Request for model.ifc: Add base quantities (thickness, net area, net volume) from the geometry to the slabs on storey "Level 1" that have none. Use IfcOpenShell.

First a look at what the model holds.

```python
import ifcopenshell
import ifcopenshell.util.element
import ifcopenshell.util.unit

model = ifcopenshell.open("model.ifc")
print(model.schema)
for unit_type in ("LENGTHUNIT", "AREAUNIT", "VOLUMEUNIT"):
    print(unit_type, ifcopenshell.util.unit.calculate_unit_scale(model, unit_type))
storey = next(s for s in model.by_type("IfcBuildingStorey") if s.Name == "Level 1")
slabs = [e for e in ifcopenshell.util.element.get_decomposition(storey) if e.is_a("IfcSlab")]
for e in sorted(slabs, key=lambda e: e.id()):
    print(e.id(), e.is_a(), e.Name, list(ifcopenshell.util.element.get_psets(e, qtos_only=True)), sep=" | ")
```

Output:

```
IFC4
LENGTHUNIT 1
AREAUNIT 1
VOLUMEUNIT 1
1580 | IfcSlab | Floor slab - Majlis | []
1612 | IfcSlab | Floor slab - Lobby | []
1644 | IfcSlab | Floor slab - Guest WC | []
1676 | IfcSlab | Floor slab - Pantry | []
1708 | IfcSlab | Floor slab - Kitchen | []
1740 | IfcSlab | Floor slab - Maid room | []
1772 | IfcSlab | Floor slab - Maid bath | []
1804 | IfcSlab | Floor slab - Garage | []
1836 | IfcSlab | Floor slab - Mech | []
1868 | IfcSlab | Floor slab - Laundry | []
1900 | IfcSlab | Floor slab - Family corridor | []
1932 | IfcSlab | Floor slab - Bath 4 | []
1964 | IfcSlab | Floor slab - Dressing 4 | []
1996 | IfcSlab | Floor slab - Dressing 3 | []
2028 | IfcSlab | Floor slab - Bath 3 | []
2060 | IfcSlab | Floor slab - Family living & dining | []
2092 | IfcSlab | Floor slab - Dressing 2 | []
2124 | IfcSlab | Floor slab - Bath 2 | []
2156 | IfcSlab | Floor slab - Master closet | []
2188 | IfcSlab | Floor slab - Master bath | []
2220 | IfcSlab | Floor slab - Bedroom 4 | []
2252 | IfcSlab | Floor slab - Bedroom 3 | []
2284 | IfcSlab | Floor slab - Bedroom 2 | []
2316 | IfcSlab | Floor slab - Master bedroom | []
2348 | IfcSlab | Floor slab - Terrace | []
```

```python
import ifcopenshell
import ifcopenshell.api.pset
import ifcopenshell.geom
import ifcopenshell.util.element
import ifcopenshell.util.shape
import ifcopenshell.util.unit

model = ifcopenshell.open("model.ifc")
unit_scale = ifcopenshell.util.unit.calculate_unit_scale(model)
area_scale = ifcopenshell.util.unit.calculate_unit_scale(model, "AREAUNIT")
volume_scale = ifcopenshell.util.unit.calculate_unit_scale(model, "VOLUMEUNIT")
settings = ifcopenshell.geom.settings()

storey = next(s for s in model.by_type("IfcBuildingStorey") if s.Name == "Level 1")
slabs = [e for e in ifcopenshell.util.element.get_decomposition(storey) if e.is_a("IfcSlab")]

for e in sorted(slabs, key=lambda e: e.id()):
    if ifcopenshell.util.element.get_psets(e, qtos_only=True, should_inherit=False):
        continue
    # Geometry comes back in metres, in the element's own axes.
    shape = ifcopenshell.geom.create_shape(settings, e)
    values = {
        "Width": ifcopenshell.util.shape.get_z(shape.geometry) / unit_scale,
        "NetArea": ifcopenshell.util.shape.get_footprint_area(shape.geometry) / area_scale,
        "NetVolume": ifcopenshell.util.shape.get_volume(shape.geometry) / volume_scale,
    }
    qto = ifcopenshell.api.pset.add_qto(model, product=e, name="Qto_SlabBaseQuantities")
    ifcopenshell.api.pset.edit_qto(model, qto=qto, properties=values)
    print(e.id(), {k: round(v, 3) for k, v in values.items()})

model.write("model_updated.ifc")
```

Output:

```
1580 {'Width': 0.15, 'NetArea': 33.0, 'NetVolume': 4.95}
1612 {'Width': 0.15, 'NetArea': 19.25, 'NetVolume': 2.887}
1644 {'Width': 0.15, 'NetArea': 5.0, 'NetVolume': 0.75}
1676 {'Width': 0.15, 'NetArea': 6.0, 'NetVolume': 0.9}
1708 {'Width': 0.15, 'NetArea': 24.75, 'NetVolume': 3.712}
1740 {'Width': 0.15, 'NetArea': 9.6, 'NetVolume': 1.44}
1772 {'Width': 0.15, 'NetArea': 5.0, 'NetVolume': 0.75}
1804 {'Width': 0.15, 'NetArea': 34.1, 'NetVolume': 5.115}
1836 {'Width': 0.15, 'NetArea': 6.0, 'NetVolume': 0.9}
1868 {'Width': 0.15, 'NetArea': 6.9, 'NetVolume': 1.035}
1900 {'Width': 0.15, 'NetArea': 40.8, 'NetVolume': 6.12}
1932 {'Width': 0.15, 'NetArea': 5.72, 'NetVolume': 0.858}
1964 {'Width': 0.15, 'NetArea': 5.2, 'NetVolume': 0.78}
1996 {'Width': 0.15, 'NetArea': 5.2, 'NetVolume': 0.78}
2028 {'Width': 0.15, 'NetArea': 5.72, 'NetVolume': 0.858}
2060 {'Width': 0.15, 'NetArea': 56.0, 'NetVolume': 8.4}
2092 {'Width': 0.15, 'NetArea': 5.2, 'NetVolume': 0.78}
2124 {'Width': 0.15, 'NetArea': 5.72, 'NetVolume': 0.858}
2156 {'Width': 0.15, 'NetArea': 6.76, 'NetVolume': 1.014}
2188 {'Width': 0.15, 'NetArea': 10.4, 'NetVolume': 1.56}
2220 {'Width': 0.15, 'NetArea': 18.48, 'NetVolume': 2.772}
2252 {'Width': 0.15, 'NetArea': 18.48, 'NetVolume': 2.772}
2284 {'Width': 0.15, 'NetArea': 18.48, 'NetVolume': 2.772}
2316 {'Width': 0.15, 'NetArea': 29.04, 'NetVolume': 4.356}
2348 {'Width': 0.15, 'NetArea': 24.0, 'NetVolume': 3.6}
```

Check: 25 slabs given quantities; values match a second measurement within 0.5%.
